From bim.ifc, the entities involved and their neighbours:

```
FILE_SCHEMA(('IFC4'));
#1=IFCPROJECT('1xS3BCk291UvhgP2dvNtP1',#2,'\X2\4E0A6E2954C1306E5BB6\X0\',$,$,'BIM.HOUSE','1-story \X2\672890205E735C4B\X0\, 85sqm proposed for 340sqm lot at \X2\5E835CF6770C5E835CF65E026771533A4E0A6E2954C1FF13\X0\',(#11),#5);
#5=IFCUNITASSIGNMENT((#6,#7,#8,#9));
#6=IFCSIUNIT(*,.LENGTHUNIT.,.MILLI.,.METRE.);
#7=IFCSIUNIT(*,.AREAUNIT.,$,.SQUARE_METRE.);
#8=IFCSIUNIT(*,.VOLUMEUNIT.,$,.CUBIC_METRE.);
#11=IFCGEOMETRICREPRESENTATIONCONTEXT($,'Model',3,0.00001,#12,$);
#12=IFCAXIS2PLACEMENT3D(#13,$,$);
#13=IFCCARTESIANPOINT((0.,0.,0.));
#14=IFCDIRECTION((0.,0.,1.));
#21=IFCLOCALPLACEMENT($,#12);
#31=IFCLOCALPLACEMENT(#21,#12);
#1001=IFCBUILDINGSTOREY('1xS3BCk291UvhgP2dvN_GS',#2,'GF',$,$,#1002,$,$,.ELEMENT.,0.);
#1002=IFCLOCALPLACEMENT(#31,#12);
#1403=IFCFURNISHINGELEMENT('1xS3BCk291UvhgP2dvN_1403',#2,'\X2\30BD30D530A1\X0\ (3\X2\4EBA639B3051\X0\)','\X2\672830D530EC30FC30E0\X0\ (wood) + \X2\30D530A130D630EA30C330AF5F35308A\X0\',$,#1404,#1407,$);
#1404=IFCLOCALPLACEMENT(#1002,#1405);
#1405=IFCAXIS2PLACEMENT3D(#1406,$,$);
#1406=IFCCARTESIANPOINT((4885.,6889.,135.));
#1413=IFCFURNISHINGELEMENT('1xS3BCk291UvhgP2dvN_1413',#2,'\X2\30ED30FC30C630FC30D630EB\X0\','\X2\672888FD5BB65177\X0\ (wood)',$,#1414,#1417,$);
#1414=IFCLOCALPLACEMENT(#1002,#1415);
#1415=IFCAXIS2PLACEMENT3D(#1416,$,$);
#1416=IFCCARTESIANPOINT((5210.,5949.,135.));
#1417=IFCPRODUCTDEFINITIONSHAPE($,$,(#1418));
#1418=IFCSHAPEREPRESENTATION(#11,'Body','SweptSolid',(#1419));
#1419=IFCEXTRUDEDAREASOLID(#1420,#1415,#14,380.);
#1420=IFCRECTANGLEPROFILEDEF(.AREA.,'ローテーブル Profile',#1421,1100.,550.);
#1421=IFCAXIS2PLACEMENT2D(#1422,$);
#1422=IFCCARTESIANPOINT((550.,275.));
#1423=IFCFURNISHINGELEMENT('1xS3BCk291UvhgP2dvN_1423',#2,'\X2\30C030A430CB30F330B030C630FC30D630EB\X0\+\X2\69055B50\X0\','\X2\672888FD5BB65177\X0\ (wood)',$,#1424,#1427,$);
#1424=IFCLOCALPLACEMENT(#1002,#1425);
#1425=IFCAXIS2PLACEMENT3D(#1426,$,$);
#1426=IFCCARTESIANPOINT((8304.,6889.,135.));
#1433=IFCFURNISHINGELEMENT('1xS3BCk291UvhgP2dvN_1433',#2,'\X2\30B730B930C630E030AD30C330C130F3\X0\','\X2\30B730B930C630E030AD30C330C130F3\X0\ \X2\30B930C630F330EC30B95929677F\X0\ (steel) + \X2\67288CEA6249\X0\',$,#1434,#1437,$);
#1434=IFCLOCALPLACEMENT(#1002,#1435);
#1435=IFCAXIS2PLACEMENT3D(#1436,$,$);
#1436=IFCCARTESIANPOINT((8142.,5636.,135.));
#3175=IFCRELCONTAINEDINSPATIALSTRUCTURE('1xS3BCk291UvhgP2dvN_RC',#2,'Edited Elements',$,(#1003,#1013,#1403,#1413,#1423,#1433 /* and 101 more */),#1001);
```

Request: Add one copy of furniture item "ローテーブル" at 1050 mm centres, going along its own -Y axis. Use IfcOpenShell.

```python
import ifcopenshell
import ifcopenshell.api.geometry
import ifcopenshell.api.root
import ifcopenshell.util.element
import ifcopenshell.util.placement
import ifcopenshell.util.unit

model = ifcopenshell.open("bim.ifc")
unit_scale = ifcopenshell.util.unit.calculate_unit_scale(model)


def reuse_history(source, copy):
    """copy_class also copies each property set's owner history, people and application; keep the originals."""
    for rel in copy.IsDefinedBy:
        if rel.is_a("IfcRelDefinesByProperties") and (history := rel.RelatingPropertyDefinition.OwnerHistory):
            rel.RelatingPropertyDefinition.OwnerHistory = source.OwnerHistory
            ifcopenshell.util.element.remove_deep2(model, history)


source = model.by_guid("1xS3BCk291UvhgP2dvN_1413")
base = ifcopenshell.util.placement.get_local_placement(source.ObjectPlacement)
step = -base[:3, 1] * 1.05 / unit_scale

for i in range(1, 2):
    copy = ifcopenshell.api.root.copy_class(model, product=source)
    copy.Representation = ifcopenshell.util.element.copy_deep(
        model, source.Representation, exclude=["IfcGeometricRepresentationContext", "IfcRepresentationMap"]
    )
    reuse_history(source, copy)
    matrix = base.copy()
    matrix[:3, 3] += i * step
    print("added at", matrix[:3, 3].round(3) + 0.0)
    ifcopenshell.api.geometry.edit_object_placement(model, product=copy, matrix=matrix, is_si=False)

model.write("bim_edited.ifc")
```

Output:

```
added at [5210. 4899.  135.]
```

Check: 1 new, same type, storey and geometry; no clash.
